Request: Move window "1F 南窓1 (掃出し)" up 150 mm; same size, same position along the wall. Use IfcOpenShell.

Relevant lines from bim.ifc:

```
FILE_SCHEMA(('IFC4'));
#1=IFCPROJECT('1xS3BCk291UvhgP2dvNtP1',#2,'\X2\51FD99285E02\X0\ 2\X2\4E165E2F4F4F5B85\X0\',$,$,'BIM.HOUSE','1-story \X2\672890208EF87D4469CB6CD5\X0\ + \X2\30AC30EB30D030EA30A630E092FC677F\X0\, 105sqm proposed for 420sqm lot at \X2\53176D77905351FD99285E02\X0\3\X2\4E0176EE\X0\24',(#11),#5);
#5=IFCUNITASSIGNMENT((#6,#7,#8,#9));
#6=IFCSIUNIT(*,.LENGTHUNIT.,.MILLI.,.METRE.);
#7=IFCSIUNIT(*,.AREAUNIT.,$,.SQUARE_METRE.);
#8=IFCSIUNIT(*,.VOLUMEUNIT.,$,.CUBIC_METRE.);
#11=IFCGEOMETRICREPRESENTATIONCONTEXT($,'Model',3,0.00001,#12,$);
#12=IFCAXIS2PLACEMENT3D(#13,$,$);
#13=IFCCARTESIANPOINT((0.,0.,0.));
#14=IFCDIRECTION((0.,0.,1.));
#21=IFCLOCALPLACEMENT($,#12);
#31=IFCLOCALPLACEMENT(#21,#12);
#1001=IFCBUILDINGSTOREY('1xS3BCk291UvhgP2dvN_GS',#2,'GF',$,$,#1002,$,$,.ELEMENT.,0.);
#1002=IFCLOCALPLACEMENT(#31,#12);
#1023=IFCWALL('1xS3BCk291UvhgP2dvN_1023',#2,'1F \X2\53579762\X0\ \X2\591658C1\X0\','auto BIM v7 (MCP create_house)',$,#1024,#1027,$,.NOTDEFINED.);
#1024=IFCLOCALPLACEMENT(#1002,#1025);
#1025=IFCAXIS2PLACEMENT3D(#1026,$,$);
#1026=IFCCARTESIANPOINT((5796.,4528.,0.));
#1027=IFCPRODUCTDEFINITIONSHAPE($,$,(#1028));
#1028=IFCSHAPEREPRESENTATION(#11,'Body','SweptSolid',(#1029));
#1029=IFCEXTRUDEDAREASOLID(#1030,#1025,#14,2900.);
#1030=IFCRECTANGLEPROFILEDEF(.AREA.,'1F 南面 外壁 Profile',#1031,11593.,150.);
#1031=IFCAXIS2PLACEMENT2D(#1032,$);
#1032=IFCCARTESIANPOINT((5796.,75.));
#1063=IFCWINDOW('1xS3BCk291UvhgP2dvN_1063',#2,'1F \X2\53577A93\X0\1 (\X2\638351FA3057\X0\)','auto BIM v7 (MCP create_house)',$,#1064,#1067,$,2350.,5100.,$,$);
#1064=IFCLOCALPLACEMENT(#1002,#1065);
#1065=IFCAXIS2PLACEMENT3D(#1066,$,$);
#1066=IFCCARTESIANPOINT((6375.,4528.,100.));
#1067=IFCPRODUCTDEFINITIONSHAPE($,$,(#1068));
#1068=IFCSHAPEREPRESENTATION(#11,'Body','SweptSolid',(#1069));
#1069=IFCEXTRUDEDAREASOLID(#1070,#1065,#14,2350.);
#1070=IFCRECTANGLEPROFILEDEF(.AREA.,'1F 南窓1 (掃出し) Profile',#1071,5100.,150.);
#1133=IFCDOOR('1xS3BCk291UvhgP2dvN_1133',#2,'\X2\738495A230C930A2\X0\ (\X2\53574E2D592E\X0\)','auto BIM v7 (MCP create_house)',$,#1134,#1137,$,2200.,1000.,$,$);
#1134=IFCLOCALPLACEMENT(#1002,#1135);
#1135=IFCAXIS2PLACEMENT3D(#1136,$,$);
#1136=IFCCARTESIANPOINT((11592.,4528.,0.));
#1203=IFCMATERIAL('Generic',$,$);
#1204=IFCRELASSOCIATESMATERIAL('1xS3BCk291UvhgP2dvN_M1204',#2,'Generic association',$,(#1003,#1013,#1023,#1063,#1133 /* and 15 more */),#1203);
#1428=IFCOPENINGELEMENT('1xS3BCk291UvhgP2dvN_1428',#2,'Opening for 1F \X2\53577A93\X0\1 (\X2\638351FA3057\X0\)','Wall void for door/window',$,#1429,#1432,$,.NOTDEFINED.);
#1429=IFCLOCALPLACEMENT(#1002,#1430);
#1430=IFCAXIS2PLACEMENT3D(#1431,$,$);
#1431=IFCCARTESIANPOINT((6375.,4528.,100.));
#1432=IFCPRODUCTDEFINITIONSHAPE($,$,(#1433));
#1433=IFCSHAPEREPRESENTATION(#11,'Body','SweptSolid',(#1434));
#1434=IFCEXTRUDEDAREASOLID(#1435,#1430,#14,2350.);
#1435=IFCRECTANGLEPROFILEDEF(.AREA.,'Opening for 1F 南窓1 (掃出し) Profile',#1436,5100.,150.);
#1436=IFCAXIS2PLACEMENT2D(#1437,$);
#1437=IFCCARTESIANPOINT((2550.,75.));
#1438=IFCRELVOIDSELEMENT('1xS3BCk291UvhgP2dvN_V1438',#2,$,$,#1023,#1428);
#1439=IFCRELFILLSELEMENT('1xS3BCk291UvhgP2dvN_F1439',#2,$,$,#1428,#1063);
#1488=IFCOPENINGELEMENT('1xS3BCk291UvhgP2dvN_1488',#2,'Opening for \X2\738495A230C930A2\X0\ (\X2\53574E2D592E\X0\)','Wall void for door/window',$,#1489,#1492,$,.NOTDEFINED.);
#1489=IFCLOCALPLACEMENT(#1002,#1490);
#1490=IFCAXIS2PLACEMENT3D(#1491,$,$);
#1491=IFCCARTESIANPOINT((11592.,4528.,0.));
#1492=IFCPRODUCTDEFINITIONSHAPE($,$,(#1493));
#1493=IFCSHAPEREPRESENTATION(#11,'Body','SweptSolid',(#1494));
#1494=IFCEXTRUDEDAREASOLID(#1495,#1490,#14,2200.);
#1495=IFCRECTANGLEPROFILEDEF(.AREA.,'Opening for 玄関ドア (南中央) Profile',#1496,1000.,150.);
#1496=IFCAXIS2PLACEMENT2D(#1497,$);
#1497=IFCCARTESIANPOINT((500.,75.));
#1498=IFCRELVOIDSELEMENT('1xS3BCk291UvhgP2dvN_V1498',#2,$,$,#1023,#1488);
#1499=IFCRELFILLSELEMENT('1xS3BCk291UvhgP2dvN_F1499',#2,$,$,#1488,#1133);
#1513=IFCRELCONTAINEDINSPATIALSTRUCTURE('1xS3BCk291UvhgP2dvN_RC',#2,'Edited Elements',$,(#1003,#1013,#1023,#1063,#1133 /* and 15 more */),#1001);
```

```python
import numpy as np
import ifcopenshell
import ifcopenshell.api.geometry
import ifcopenshell.util.placement
import ifcopenshell.util.unit

model = ifcopenshell.open("bim.ifc")
unit_scale = ifcopenshell.util.unit.calculate_unit_scale(model)

window = model.by_id(1063)
opening = window.FillsVoids[0].RelatingOpeningElement
dz = 150.0

shift = np.array([0.0, 0.0, dz])
# The window is not placed relative to its opening, so move both.
for product in (opening, window):
    matrix = ifcopenshell.util.placement.get_local_placement(product.ObjectPlacement)
    matrix[:3, 3] += shift
    ifcopenshell.api.geometry.edit_object_placement(model, product=product, matrix=matrix, is_si=False)

print(f"moved by {dz * unit_scale:+.3f} m")

model.write("bim-out.ifc")
```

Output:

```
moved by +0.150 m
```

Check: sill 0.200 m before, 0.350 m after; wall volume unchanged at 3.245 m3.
